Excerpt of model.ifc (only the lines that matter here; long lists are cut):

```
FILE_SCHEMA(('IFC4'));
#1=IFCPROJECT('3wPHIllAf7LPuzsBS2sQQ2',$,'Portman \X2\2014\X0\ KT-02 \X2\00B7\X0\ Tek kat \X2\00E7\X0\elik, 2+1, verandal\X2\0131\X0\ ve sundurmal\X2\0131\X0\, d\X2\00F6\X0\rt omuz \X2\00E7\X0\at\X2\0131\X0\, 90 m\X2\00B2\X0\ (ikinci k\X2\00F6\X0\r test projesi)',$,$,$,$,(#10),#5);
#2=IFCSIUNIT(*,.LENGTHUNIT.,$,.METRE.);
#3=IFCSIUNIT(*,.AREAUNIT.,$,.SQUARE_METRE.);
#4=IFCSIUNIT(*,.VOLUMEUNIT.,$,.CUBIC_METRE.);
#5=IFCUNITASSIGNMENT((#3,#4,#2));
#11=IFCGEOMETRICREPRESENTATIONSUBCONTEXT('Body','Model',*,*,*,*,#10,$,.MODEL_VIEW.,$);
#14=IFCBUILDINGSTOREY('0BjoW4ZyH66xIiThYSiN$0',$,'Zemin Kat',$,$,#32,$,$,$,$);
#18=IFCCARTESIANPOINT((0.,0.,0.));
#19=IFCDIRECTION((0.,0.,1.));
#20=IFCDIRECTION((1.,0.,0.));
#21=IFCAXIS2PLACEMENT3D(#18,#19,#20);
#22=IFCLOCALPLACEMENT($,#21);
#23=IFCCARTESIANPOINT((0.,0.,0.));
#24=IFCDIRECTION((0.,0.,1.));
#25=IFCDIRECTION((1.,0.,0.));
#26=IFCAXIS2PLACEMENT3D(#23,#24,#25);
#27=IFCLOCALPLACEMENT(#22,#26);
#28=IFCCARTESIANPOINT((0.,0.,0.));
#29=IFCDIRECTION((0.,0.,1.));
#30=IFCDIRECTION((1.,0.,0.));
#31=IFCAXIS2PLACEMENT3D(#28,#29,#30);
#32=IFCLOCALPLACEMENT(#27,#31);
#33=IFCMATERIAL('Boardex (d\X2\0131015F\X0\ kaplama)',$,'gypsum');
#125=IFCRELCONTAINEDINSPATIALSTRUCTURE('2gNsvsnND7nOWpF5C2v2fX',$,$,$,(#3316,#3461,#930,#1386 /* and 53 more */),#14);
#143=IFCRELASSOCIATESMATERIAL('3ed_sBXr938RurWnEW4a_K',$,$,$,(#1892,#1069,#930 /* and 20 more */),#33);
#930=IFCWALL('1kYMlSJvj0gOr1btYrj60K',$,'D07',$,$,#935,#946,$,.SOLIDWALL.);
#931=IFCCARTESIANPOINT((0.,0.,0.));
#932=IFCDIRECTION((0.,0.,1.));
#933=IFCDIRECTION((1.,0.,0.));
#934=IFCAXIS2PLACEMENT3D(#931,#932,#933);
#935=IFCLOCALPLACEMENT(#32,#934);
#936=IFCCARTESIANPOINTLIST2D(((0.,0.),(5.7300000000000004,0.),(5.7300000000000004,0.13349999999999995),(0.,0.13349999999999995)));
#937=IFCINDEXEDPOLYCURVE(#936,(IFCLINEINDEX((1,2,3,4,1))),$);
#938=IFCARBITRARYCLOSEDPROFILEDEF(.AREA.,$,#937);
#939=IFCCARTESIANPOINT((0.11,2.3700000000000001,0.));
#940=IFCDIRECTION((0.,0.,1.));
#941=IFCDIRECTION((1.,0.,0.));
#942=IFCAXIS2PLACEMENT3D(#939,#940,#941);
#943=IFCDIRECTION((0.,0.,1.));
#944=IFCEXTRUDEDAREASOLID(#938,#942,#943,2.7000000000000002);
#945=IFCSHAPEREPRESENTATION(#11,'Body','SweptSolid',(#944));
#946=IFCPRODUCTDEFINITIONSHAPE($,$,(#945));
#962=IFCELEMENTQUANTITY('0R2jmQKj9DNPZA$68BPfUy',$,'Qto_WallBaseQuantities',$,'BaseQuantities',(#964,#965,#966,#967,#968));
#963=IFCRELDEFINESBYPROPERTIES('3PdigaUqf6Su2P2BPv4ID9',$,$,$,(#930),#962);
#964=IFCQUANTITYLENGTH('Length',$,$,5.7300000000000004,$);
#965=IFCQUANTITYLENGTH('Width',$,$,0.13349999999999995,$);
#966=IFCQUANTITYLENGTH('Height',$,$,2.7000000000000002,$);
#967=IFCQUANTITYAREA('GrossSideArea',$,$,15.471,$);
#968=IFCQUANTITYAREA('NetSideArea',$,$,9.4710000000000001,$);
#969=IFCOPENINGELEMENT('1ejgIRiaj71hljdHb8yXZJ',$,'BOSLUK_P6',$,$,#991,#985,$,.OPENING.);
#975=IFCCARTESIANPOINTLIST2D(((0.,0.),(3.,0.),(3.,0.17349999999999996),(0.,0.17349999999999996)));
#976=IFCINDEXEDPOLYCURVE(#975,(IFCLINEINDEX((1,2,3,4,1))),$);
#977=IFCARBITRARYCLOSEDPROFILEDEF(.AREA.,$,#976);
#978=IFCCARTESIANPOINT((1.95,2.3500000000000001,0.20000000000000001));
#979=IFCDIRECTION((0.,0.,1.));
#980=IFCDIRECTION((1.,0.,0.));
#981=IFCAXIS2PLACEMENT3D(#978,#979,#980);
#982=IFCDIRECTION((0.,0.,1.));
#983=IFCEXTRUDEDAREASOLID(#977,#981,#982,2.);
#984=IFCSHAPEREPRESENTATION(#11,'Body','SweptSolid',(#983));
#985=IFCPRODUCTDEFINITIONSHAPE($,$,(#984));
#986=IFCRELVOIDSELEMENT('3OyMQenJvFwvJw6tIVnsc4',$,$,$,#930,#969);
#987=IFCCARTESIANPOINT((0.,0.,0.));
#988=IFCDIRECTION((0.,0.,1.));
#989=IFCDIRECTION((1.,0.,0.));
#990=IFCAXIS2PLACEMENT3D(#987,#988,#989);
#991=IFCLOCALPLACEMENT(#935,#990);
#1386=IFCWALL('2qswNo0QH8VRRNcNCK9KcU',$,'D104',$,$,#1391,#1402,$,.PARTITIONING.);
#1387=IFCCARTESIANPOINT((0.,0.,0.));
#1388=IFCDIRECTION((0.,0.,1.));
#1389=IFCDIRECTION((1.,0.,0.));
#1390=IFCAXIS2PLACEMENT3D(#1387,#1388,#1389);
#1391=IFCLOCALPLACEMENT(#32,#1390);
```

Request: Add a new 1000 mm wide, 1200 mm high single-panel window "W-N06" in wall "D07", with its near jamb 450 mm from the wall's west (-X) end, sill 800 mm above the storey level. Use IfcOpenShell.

```python
import numpy as np
import ifcopenshell
import ifcopenshell.api.feature
import ifcopenshell.api.geometry
import ifcopenshell.api.pset
import ifcopenshell.api.root
import ifcopenshell.api.spatial
import ifcopenshell.geom
import ifcopenshell.util.element
import ifcopenshell.util.placement
import ifcopenshell.util.representation
import ifcopenshell.util.shape
import ifcopenshell.util.unit

model = ifcopenshell.open("model.ifc")
unit_scale = ifcopenshell.util.unit.calculate_unit_scale(model)
area_scale = ifcopenshell.util.unit.calculate_unit_scale(model, "AREAUNIT")
settings = ifcopenshell.geom.settings()


def volume(element):
    """Net volume in cubic metres, openings subtracted."""
    shape = ifcopenshell.geom.create_shape(settings, element)
    return ifcopenshell.util.shape.get_volume(shape.geometry)


wall = model.by_id(930)
storey = ifcopenshell.util.element.get_container(wall, ifc_class="IfcBuildingStorey")
context = ifcopenshell.util.representation.get_context(model, "Model", "Body", "MODEL_VIEW")
before = volume(wall)

width, height, from_end, sill = 1, 1.2, 0.45, 0.8  # metres

# The wall runs along its own X axis, and the end named is its -X end.
wall_shape = ifcopenshell.geom.create_shape(settings, wall)
x, y, z = ifcopenshell.util.shape.get_vertices(wall_shape.geometry).T
start = x.min() + from_end
face, thickness = float(y.min()), float(y.max() - y.min())
wall_matrix = ifcopenshell.util.placement.get_local_placement(wall.ObjectPlacement)
level = ifcopenshell.util.placement.get_local_placement(storey.ObjectPlacement)[2, 3]


def in_wall(x, y):
    """Placement at x, y metres in the wall's axes, at sill height."""
    matrix = wall_matrix.copy()
    matrix[:, 3] = wall_matrix @ np.array([x / unit_scale, y / unit_scale, 0.0, 1.0])
    matrix[2, 3] = level + sill / unit_scale
    return matrix


# Opening: a box that overshoots both wall faces by 50 mm.
opening = ifcopenshell.api.root.create_entity(model, ifc_class="IfcOpeningElement", predefined_type="OPENING")
box = ifcopenshell.api.geometry.add_wall_representation(
    model, context=context, length=width, height=height, thickness=thickness + 0.1
)
ifcopenshell.api.geometry.assign_representation(model, product=opening, representation=box)
ifcopenshell.api.geometry.edit_object_placement(model, product=opening, matrix=in_wall(start, face - 0.05), is_si=False)
ifcopenshell.api.feature.add_feature(model, feature=opening, element=wall)

window = ifcopenshell.api.root.create_entity(model, ifc_class="IfcWindow", name="W-N06", predefined_type="WINDOW")
window.OverallWidth, window.OverallHeight = width / unit_scale, height / unit_scale
window.PartitioningType = "SINGLE_PANEL"
body = ifcopenshell.api.geometry.add_window_representation(
    model,
    context=context,
    overall_width=window.OverallWidth,
    overall_height=window.OverallHeight,
    partition_type="SINGLE_PANEL",
)
ifcopenshell.api.geometry.assign_representation(model, product=window, representation=body)
ifcopenshell.api.spatial.assign_container(model, products=[window], relating_structure=storey)
ifcopenshell.api.feature.add_filling(model, opening=opening, element=window)

# Centre the window in the wall's thickness.
ifcopenshell.api.geometry.edit_object_placement(model, product=window, matrix=in_wall(start, face), is_si=False)
window_shape = ifcopenshell.geom.create_shape(settings, window)
depth = ifcopenshell.util.shape.get_vertices(window_shape.geometry)[:, 1]
offset = face + thickness / 2 - (depth.min() + depth.max()) / 2
ifcopenshell.api.geometry.edit_object_placement(model, product=window, matrix=in_wall(start, offset), is_si=False)

after = volume(wall)

# Update the wall's stored quantities.
qto = model.by_id(ifcopenshell.util.element.get_pset(wall, "Qto_WallBaseQuantities", should_inherit=False)["id"])
ifcopenshell.api.pset.edit_qto(model, qto=qto, properties={"NetSideArea": after / thickness / area_scale})

print(f"wall volume {before:.3f} -> {after:.3f} m3")

model.write("model_edited.ifc")
```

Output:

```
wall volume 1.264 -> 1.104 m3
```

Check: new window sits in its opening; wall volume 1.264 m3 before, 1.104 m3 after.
